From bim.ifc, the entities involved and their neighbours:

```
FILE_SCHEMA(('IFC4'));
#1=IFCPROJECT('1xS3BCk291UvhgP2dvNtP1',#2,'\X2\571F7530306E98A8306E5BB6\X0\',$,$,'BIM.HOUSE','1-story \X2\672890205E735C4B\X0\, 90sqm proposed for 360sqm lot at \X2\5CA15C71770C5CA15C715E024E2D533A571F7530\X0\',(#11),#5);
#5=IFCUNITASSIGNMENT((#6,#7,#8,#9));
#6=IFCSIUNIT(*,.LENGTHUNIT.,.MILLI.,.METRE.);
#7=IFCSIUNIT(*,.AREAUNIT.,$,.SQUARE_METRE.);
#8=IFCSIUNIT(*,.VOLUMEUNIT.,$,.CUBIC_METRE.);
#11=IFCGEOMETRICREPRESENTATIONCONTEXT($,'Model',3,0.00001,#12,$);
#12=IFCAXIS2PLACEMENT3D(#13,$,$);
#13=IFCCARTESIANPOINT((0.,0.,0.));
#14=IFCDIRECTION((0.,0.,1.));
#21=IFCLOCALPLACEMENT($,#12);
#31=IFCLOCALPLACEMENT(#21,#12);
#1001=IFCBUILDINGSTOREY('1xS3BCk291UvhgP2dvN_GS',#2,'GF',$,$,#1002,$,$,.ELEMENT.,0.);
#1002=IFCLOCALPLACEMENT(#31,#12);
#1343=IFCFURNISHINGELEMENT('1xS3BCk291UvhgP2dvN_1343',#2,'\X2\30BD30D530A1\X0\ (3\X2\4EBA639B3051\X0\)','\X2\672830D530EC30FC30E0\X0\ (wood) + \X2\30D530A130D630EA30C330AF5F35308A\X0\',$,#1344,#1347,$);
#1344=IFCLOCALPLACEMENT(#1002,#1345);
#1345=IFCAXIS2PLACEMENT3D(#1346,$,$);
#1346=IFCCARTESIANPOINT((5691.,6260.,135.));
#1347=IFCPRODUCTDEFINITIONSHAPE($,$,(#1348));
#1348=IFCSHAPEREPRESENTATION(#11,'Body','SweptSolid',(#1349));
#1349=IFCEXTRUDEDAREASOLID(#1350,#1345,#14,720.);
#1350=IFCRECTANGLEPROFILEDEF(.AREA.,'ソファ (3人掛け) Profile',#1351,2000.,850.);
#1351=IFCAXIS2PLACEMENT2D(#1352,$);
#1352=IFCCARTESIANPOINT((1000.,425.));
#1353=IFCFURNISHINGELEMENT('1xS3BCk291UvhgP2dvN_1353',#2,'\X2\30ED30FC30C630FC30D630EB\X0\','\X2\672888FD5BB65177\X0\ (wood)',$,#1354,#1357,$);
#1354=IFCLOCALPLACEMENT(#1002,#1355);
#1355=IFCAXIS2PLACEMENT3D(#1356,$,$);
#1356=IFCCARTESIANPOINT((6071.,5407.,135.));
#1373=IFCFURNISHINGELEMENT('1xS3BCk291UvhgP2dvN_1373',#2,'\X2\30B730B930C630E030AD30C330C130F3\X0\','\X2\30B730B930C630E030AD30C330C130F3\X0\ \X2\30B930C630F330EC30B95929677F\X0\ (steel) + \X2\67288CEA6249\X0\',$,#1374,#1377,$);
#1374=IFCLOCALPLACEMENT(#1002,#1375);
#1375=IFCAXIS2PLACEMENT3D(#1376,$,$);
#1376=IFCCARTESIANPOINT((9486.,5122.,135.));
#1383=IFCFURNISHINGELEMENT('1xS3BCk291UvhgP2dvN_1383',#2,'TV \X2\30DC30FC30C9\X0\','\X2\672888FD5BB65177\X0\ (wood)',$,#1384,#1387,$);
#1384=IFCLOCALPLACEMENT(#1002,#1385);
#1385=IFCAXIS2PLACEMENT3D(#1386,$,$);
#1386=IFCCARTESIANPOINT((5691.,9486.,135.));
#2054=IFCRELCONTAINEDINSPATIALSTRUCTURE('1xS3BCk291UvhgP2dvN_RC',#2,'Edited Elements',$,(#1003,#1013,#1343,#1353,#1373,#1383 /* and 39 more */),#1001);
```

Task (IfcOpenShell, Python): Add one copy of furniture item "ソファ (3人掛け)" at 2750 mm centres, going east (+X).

```python
import numpy as np
import ifcopenshell
import ifcopenshell.api.geometry
import ifcopenshell.api.root
import ifcopenshell.util.element
import ifcopenshell.util.placement
import ifcopenshell.util.unit

model = ifcopenshell.open("bim.ifc")
unit_scale = ifcopenshell.util.unit.calculate_unit_scale(model)


def reuse_history(source, copy):
    """copy_class also copies each property set's owner history, people and application; keep the originals."""
    for rel in copy.IsDefinedBy:
        if rel.is_a("IfcRelDefinesByProperties") and (history := rel.RelatingPropertyDefinition.OwnerHistory):
            rel.RelatingPropertyDefinition.OwnerHistory = source.OwnerHistory
            ifcopenshell.util.element.remove_deep2(model, history)


source = model.by_guid("1xS3BCk291UvhgP2dvN_1343")
base = ifcopenshell.util.placement.get_local_placement(source.ObjectPlacement)
step = np.array([1.0, 0.0, 0.0]) * 2.75 / unit_scale

for i in range(1, 2):
    copy = ifcopenshell.api.root.copy_class(model, product=source)
    copy.Representation = ifcopenshell.util.element.copy_deep(
        model, source.Representation, exclude=["IfcGeometricRepresentationContext", "IfcRepresentationMap"]
    )
    reuse_history(source, copy)
    matrix = base.copy()
    matrix[:3, 3] += i * step
    print("added at", matrix[:3, 3].round(3) + 0.0)
    ifcopenshell.api.geometry.edit_object_placement(model, product=copy, matrix=matrix, is_si=False)

model.write("bim_updated.ifc")
```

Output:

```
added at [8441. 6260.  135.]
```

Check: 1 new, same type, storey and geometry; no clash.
